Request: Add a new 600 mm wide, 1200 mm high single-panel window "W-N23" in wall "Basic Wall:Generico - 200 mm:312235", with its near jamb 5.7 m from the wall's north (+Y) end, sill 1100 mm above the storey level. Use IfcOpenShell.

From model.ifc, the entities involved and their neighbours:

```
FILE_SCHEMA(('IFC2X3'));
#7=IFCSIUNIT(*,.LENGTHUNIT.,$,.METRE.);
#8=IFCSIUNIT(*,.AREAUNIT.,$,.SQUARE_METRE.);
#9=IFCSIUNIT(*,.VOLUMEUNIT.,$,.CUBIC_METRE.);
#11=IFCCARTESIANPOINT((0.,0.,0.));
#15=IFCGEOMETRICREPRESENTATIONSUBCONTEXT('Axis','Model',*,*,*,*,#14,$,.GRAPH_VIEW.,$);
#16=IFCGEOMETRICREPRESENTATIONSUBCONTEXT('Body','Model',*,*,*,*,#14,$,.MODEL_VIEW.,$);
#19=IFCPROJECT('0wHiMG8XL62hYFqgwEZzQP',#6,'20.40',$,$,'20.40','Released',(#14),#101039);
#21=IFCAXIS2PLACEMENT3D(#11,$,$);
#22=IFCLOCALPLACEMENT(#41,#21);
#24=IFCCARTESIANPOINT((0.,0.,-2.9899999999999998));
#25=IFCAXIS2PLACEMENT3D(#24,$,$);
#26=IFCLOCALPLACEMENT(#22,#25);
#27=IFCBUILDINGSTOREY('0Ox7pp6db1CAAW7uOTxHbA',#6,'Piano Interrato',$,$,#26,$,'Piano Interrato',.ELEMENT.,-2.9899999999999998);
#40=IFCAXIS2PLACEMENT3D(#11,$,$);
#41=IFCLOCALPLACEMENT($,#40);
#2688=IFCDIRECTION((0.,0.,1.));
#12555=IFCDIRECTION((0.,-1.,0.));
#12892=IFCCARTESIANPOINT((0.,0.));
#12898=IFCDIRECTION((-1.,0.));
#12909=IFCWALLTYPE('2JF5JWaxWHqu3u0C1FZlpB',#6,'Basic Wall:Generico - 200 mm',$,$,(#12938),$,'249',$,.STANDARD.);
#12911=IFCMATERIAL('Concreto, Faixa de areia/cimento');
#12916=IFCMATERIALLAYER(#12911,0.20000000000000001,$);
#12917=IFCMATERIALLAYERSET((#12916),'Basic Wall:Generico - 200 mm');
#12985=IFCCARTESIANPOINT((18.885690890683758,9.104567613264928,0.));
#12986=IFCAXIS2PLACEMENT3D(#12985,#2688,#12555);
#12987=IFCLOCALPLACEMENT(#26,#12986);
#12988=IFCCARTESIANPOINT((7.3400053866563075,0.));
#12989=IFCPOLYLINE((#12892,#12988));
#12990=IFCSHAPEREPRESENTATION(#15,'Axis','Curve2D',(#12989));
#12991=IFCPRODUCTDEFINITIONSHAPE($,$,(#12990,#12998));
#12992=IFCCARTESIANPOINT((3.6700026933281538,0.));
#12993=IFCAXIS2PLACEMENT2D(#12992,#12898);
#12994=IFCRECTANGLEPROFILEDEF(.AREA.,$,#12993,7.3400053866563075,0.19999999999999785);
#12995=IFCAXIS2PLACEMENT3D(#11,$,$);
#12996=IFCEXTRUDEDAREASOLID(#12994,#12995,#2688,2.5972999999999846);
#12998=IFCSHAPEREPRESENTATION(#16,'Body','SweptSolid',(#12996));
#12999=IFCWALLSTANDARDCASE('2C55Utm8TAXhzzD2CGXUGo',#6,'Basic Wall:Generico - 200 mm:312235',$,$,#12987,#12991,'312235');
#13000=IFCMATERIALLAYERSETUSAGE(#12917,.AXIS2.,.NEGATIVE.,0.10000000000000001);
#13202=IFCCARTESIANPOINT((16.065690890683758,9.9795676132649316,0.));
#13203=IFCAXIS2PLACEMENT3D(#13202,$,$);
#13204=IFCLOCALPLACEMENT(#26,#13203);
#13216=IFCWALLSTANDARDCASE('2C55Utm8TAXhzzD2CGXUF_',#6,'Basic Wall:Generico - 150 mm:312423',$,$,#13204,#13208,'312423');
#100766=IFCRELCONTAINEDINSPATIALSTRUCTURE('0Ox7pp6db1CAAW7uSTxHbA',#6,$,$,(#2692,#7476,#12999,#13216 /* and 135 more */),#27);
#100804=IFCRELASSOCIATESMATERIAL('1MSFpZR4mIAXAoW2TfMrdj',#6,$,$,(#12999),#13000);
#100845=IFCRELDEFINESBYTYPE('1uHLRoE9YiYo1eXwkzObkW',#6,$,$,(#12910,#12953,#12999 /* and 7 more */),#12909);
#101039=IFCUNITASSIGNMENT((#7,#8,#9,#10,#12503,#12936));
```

```python
import numpy as np
import ifcopenshell
import ifcopenshell.api.feature
import ifcopenshell.api.geometry
import ifcopenshell.api.root
import ifcopenshell.api.spatial
import ifcopenshell.api.type
import ifcopenshell.geom
import ifcopenshell.util.element
import ifcopenshell.util.placement
import ifcopenshell.util.representation
import ifcopenshell.util.shape
import ifcopenshell.util.unit

model = ifcopenshell.open("model.ifc")
unit_scale = ifcopenshell.util.unit.calculate_unit_scale(model)
settings = ifcopenshell.geom.settings()


def volume(element):
    """Net volume in cubic metres, openings subtracted."""
    shape = ifcopenshell.geom.create_shape(settings, element)
    return ifcopenshell.util.shape.get_volume(shape.geometry)


wall = model.by_guid("2C55Utm8TAXhzzD2CGXUGo")
storey = ifcopenshell.util.element.get_container(wall, ifc_class="IfcBuildingStorey")
context = ifcopenshell.util.representation.get_context(model, "Model", "Body", "MODEL_VIEW")
before = volume(wall)

width, height, from_end, sill = 0.6, 1.2, 5.7, 1.1  # metres

# The wall runs along its own X axis, and the end named is its -X end.
wall_shape = ifcopenshell.geom.create_shape(settings, wall)
x, y, z = ifcopenshell.util.shape.get_vertices(wall_shape.geometry).T
start = x.min() + from_end
face, thickness = float(y.min()), float(y.max() - y.min())
wall_matrix = ifcopenshell.util.placement.get_local_placement(wall.ObjectPlacement)
level = ifcopenshell.util.placement.get_local_placement(storey.ObjectPlacement)[2, 3]


def in_wall(x, y):
    """Placement at x, y metres in the wall's axes, at sill height."""
    matrix = wall_matrix.copy()
    matrix[:, 3] = wall_matrix @ np.array([x / unit_scale, y / unit_scale, 0.0, 1.0])
    matrix[2, 3] = level + sill / unit_scale
    return matrix


# Opening: a box that overshoots both wall faces by 50 mm.
opening = ifcopenshell.api.root.create_entity(model, ifc_class="IfcOpeningElement")
box = ifcopenshell.api.geometry.add_wall_representation(
    model, context=context, length=width, height=height, thickness=thickness + 0.1
)
ifcopenshell.api.geometry.assign_representation(model, product=opening, representation=box)
ifcopenshell.api.geometry.edit_object_placement(model, product=opening, matrix=in_wall(start, face - 0.05), is_si=False)
ifcopenshell.api.feature.add_feature(model, feature=opening, element=wall)

window = ifcopenshell.api.root.create_entity(model, ifc_class="IfcWindow", name="W-N23")
window.OverallWidth, window.OverallHeight = width / unit_scale, height / unit_scale
body = ifcopenshell.api.geometry.add_window_representation(
    model,
    context=context,
    overall_width=window.OverallWidth,
    overall_height=window.OverallHeight,
    partition_type="SINGLE_PANEL",
)
ifcopenshell.api.geometry.assign_representation(model, product=window, representation=body)
ifcopenshell.api.spatial.assign_container(model, products=[window], relating_structure=storey)
fills = ifcopenshell.api.feature.add_filling(model, opening=opening, element=window)
fills.OwnerHistory = window.OwnerHistory  # required in IFC2X3

# IFC2X3 keeps the operation on the window style.
style = ifcopenshell.api.root.create_entity(model, ifc_class="IfcWindowStyle", name="W-N23")
style.OperationType, style.ConstructionType = "SINGLE_PANEL", "NOTDEFINED"
style.ParameterTakesPrecedence = style.Sizeable = False
ifcopenshell.api.type.assign_type(model, related_objects=[window], relating_type=style)

# Centre the window in the wall's thickness.
ifcopenshell.api.geometry.edit_object_placement(model, product=window, matrix=in_wall(start, face), is_si=False)
window_shape = ifcopenshell.geom.create_shape(settings, window)
depth = ifcopenshell.util.shape.get_vertices(window_shape.geometry)[:, 1]
offset = face + thickness / 2 - (depth.min() + depth.max()) / 2
ifcopenshell.api.geometry.edit_object_placement(model, product=window, matrix=in_wall(start, offset), is_si=False)

after = volume(wall)

print(f"wall volume {before:.3f} -> {after:.3f} m3")

model.write("model_rev.ifc")
```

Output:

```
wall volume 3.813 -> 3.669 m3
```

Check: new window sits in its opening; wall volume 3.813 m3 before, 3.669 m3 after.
